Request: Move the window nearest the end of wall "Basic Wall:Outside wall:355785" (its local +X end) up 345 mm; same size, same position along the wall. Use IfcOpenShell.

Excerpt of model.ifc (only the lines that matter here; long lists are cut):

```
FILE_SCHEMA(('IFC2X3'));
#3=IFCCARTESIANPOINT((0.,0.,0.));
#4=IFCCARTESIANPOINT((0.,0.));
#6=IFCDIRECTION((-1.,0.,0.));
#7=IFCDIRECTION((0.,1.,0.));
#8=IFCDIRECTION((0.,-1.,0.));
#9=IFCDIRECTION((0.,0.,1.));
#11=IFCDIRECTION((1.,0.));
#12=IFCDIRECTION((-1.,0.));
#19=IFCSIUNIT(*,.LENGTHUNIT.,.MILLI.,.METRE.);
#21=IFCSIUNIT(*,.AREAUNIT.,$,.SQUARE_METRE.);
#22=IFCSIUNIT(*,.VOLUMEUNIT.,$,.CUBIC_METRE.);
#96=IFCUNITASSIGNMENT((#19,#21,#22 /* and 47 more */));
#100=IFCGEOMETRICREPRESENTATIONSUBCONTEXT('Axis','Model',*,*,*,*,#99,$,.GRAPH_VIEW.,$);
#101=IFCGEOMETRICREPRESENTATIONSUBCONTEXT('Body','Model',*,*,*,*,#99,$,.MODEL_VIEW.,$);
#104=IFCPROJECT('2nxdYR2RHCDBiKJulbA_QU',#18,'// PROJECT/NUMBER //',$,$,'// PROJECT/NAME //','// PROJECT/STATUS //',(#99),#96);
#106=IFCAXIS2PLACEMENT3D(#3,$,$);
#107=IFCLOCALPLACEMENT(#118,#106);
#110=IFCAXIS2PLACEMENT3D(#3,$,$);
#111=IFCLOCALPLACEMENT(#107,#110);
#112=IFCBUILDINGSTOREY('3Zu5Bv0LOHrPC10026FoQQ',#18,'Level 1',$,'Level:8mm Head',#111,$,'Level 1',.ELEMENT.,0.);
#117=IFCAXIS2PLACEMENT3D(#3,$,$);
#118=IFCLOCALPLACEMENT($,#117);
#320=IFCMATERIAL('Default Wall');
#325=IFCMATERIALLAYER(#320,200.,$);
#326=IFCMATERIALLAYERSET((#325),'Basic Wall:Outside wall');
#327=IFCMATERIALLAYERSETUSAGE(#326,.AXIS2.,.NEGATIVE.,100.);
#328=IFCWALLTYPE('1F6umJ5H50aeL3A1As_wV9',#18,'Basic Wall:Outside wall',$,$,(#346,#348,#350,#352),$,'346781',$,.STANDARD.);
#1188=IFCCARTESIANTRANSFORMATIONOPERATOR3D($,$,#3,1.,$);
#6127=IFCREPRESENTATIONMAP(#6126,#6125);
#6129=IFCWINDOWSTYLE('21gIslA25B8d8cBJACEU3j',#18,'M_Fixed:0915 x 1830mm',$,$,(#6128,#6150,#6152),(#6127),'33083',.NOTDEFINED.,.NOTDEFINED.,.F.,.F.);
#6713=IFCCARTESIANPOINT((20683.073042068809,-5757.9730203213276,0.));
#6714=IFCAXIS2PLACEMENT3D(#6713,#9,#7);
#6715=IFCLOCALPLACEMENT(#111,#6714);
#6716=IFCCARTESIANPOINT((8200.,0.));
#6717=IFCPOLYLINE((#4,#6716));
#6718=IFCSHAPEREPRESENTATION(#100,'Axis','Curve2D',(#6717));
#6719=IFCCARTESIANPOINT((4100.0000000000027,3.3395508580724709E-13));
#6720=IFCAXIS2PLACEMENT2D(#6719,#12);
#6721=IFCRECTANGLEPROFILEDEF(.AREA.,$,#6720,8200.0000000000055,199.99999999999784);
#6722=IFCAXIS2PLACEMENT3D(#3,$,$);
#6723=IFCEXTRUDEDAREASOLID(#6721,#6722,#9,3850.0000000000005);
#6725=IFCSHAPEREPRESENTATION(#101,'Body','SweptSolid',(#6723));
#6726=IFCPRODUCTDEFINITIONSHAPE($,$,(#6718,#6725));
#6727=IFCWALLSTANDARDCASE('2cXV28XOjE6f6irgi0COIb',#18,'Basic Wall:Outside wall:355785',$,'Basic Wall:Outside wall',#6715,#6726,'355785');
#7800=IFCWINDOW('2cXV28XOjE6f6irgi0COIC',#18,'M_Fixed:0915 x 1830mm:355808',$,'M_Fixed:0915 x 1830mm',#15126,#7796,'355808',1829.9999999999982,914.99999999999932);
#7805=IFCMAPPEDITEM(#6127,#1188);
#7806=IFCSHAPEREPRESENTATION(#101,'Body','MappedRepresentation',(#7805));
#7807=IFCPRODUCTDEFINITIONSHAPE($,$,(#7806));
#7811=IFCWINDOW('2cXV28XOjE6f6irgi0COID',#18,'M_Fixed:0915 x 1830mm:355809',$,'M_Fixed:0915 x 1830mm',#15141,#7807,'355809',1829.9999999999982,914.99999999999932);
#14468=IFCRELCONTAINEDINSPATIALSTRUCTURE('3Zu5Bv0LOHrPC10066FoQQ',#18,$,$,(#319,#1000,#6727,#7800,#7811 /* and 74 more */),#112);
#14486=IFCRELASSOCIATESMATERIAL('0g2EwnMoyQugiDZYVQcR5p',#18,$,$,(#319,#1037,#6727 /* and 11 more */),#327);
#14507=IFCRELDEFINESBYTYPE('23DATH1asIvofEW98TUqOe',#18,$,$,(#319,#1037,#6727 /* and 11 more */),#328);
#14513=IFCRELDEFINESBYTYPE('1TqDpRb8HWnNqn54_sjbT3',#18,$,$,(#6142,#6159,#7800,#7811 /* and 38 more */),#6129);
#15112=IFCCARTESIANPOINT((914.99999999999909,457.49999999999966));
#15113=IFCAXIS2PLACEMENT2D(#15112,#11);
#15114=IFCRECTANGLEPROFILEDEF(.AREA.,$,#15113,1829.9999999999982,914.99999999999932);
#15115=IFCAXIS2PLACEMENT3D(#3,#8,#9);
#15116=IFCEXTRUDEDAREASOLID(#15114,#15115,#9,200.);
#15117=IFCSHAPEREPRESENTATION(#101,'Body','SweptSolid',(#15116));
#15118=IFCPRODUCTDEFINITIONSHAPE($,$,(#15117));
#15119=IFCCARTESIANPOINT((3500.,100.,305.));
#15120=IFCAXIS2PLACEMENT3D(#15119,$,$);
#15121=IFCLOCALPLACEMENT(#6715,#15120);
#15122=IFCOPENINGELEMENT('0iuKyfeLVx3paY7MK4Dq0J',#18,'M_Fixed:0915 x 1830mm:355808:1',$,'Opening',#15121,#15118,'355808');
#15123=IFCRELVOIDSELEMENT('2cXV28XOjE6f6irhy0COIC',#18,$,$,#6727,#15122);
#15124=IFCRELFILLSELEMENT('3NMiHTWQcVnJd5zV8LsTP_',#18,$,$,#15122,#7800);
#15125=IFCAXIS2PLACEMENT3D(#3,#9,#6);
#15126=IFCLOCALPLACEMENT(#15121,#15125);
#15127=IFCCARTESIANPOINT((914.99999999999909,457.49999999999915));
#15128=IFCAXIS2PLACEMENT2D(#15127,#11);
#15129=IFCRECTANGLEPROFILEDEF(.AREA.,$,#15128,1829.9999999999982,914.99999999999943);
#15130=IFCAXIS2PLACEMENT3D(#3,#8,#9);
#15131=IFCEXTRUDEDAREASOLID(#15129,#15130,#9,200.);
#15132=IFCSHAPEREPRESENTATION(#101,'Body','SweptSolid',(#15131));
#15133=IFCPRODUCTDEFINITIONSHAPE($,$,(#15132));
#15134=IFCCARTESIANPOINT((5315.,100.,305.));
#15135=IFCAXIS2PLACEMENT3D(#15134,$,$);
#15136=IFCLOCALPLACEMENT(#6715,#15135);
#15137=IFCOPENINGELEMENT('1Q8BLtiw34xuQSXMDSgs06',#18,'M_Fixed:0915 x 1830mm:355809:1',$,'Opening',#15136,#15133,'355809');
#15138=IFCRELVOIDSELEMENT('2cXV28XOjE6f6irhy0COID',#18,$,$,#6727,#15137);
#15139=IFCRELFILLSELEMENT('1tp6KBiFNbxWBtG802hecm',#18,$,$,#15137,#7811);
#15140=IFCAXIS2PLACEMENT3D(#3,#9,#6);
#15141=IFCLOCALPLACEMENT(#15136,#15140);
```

```python
import numpy as np
import ifcopenshell
import ifcopenshell.api.geometry
import ifcopenshell.util.placement
import ifcopenshell.util.unit

model = ifcopenshell.open("model.ifc")
unit_scale = ifcopenshell.util.unit.calculate_unit_scale(model)

window = model.by_guid("2cXV28XOjE6f6irgi0COID")
opening = window.FillsVoids[0].RelatingOpeningElement
dz = 0.345 / unit_scale

shift = np.array([0.0, 0.0, dz])
# The window is placed relative to its opening, so it follows when the opening moves.
matrix = ifcopenshell.util.placement.get_local_placement(opening.ObjectPlacement)
matrix[:3, 3] += shift
ifcopenshell.api.geometry.edit_object_placement(
    model, product=opening, matrix=matrix, is_si=False, should_transform_children=True
)

print(f"moved by {dz * unit_scale:+.3f} m")

model.write("model_v2.ifc")
```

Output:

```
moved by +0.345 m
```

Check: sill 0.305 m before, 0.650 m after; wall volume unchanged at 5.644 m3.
